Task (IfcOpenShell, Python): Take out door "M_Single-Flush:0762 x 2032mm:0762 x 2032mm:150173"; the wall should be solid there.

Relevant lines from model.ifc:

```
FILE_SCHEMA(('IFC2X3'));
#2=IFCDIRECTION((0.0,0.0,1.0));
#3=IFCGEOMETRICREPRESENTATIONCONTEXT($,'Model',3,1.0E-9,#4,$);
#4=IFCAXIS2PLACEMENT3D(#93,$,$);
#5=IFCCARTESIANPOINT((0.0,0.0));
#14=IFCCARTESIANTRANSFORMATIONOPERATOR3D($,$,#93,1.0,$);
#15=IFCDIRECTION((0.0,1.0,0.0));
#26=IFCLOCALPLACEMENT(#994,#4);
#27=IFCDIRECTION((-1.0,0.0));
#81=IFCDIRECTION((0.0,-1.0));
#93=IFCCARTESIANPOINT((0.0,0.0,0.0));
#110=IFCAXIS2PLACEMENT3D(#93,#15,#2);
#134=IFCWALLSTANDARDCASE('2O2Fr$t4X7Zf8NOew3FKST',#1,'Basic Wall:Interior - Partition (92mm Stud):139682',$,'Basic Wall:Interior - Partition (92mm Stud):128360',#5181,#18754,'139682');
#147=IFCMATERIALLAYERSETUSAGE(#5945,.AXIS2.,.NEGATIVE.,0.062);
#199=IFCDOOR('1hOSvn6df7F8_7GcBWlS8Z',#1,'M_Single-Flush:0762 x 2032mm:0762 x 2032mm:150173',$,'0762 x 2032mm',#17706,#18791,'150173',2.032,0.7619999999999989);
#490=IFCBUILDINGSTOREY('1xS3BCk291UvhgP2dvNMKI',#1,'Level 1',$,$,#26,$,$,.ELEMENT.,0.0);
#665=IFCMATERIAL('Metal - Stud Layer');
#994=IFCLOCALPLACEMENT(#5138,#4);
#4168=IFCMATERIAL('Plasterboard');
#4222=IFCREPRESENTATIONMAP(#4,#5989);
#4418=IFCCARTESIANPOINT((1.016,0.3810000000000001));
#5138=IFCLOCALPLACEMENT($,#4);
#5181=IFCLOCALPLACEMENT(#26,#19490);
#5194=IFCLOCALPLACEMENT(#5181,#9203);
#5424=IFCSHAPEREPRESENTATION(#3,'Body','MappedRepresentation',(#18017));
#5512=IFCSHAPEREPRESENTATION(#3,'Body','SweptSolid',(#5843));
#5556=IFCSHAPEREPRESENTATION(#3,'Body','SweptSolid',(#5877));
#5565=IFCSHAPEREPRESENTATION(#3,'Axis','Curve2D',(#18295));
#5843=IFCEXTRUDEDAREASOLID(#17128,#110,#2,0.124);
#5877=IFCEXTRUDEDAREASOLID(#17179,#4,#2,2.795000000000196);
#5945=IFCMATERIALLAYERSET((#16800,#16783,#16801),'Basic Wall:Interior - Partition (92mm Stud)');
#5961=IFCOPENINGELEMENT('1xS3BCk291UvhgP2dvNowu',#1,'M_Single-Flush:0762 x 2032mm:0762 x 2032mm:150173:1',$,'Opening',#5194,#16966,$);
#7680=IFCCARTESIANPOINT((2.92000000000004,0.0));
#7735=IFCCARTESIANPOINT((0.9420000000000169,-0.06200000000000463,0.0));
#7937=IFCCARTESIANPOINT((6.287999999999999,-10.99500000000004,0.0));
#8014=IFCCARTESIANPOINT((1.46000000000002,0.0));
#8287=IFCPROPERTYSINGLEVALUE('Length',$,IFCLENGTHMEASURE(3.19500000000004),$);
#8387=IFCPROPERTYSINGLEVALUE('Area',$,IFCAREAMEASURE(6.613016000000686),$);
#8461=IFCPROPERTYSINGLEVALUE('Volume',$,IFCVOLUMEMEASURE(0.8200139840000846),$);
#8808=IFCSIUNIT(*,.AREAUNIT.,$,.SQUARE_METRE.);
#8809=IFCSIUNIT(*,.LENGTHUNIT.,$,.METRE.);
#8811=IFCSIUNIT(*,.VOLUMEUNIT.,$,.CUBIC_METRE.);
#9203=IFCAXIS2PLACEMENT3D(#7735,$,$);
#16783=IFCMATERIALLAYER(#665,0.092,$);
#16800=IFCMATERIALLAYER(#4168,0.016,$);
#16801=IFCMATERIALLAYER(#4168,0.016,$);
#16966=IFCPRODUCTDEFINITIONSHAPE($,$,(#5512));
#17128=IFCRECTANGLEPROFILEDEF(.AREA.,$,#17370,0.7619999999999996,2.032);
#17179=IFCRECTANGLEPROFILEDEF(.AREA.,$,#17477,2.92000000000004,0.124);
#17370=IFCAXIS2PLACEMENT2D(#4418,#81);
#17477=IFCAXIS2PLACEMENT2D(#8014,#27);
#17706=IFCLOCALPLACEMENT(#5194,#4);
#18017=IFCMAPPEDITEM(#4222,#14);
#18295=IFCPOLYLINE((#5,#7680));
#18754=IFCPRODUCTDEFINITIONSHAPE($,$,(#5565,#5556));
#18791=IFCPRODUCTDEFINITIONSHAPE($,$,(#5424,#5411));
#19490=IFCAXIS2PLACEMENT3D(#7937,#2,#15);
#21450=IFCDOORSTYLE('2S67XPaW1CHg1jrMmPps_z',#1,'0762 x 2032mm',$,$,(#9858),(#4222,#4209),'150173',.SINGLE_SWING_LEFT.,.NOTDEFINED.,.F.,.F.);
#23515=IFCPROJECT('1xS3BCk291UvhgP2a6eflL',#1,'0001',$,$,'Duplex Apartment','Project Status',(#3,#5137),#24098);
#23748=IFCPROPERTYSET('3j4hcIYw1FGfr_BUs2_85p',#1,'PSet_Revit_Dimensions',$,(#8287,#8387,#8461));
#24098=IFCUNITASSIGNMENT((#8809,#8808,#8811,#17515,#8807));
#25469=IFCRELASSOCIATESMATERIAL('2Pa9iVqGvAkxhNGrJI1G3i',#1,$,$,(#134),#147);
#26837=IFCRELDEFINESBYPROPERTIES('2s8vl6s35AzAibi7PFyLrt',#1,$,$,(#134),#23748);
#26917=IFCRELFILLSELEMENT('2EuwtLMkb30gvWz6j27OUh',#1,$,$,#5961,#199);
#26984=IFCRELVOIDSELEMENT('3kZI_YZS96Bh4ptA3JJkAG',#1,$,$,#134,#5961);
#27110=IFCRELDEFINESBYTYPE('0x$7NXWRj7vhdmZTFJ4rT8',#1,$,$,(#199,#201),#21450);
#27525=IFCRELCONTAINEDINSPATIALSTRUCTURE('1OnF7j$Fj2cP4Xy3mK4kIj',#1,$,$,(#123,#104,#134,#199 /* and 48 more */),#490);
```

```python
import ifcopenshell
import ifcopenshell.api.feature
import ifcopenshell.api.pset
import ifcopenshell.api.root
import ifcopenshell.geom
import ifcopenshell.util.element
import ifcopenshell.util.shape
import ifcopenshell.util.unit

model = ifcopenshell.open("model.ifc")
area_scale = ifcopenshell.util.unit.calculate_unit_scale(model, "AREAUNIT")
volume_scale = ifcopenshell.util.unit.calculate_unit_scale(model, "VOLUMEUNIT")
settings = ifcopenshell.geom.settings()


def volume(element):
    """Net volume in cubic metres, openings subtracted."""
    shape = ifcopenshell.geom.create_shape(settings, element)
    return ifcopenshell.util.shape.get_volume(shape.geometry)


door = model.by_id(199)
opening = door.FillsVoids[0].RelatingOpeningElement
wall = opening.VoidsElements[0].RelatingBuildingElement
before = volume(wall)

ifcopenshell.api.root.remove_product(model, product=door)
ifcopenshell.api.feature.remove_feature(model, feature=opening)

after = volume(wall)
thickness = 0.124  # wall thickness in metres

# Update the wall's stored quantities.
pset = model.by_id(ifcopenshell.util.element.get_pset(wall, "PSet_Revit_Dimensions", should_inherit=False)["id"])
ifcopenshell.api.pset.edit_pset(model, pset=pset, properties={
    "Area": model.create_entity("IfcAreaMeasure", after / thickness / area_scale),
    "Volume": model.create_entity("IfcVolumeMeasure", after / volume_scale),
})

print(f"wall volume {before:.3f} -> {after:.3f} m3")

model.write("model-out.ifc")
```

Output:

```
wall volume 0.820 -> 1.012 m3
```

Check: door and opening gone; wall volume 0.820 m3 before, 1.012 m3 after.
